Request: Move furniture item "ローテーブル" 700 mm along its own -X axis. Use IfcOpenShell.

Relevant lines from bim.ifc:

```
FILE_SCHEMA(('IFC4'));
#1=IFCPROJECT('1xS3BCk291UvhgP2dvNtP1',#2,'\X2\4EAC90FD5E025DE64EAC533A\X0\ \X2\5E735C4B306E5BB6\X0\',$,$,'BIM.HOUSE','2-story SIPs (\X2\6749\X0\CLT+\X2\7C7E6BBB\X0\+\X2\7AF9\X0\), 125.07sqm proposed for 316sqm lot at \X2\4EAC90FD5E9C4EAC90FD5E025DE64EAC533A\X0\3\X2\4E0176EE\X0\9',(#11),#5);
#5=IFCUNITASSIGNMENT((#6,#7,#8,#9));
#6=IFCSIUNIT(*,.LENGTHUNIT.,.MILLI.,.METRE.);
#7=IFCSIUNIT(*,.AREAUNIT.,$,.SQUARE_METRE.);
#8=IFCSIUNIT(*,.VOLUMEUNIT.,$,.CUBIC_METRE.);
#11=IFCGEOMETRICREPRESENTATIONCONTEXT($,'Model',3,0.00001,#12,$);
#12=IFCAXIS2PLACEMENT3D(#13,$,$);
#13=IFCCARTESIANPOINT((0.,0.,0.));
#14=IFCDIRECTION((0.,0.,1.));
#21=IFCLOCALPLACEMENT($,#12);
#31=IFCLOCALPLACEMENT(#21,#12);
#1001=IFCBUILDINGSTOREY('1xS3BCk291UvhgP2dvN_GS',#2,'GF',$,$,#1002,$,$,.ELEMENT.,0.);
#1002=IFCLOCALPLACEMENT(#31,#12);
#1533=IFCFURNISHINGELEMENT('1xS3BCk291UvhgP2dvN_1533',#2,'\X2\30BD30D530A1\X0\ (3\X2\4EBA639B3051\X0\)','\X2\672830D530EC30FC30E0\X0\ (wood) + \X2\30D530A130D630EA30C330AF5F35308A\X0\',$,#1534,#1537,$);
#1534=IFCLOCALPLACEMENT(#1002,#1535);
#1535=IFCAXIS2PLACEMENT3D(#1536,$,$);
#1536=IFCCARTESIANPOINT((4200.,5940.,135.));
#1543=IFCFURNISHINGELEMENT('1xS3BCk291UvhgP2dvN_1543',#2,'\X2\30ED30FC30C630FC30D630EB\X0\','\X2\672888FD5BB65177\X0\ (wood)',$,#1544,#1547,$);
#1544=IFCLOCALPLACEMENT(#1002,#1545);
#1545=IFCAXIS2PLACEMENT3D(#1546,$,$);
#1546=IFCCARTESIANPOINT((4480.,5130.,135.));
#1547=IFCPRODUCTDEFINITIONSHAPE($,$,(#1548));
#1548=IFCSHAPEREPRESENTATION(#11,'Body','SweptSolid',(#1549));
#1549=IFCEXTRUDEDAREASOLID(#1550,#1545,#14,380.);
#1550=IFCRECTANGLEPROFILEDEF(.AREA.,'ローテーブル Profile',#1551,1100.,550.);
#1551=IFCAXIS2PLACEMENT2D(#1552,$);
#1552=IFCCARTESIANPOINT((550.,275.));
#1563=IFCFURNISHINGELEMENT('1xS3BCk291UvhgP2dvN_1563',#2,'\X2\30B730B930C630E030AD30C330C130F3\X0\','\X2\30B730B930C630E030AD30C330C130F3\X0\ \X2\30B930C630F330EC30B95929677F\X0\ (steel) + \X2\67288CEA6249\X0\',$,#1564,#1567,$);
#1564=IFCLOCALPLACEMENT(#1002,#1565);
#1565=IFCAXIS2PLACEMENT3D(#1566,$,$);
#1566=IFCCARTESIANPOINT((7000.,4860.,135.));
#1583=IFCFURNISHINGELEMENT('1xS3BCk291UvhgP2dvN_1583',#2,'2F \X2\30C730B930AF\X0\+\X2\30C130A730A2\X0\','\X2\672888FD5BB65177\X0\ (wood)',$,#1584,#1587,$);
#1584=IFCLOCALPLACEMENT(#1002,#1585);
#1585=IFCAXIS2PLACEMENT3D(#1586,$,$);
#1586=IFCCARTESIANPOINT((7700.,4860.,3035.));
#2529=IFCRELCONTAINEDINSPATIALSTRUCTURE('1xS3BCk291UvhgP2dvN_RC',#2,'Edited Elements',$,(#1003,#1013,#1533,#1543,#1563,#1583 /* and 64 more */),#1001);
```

```python
import ifcopenshell
import ifcopenshell.api.geometry
import ifcopenshell.util.placement
import ifcopenshell.util.unit

model = ifcopenshell.open("bim.ifc")
unit_scale = ifcopenshell.util.unit.calculate_unit_scale(model)

item = model.by_id(1543)
matrix = ifcopenshell.util.placement.get_local_placement(item.ObjectPlacement)
matrix[:3, 3] -= matrix[:3, 0] * 0.7 / unit_scale
ifcopenshell.api.geometry.edit_object_placement(model, product=item, matrix=matrix, is_si=False)

print(ifcopenshell.util.placement.get_local_placement(item.ObjectPlacement).round(3) + 0.0)

model.write("bim_updated.ifc")
```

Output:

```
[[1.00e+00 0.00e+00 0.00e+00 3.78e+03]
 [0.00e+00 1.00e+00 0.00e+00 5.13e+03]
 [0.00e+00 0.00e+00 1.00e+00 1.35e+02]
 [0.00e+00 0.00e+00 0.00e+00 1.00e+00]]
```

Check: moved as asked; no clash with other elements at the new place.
